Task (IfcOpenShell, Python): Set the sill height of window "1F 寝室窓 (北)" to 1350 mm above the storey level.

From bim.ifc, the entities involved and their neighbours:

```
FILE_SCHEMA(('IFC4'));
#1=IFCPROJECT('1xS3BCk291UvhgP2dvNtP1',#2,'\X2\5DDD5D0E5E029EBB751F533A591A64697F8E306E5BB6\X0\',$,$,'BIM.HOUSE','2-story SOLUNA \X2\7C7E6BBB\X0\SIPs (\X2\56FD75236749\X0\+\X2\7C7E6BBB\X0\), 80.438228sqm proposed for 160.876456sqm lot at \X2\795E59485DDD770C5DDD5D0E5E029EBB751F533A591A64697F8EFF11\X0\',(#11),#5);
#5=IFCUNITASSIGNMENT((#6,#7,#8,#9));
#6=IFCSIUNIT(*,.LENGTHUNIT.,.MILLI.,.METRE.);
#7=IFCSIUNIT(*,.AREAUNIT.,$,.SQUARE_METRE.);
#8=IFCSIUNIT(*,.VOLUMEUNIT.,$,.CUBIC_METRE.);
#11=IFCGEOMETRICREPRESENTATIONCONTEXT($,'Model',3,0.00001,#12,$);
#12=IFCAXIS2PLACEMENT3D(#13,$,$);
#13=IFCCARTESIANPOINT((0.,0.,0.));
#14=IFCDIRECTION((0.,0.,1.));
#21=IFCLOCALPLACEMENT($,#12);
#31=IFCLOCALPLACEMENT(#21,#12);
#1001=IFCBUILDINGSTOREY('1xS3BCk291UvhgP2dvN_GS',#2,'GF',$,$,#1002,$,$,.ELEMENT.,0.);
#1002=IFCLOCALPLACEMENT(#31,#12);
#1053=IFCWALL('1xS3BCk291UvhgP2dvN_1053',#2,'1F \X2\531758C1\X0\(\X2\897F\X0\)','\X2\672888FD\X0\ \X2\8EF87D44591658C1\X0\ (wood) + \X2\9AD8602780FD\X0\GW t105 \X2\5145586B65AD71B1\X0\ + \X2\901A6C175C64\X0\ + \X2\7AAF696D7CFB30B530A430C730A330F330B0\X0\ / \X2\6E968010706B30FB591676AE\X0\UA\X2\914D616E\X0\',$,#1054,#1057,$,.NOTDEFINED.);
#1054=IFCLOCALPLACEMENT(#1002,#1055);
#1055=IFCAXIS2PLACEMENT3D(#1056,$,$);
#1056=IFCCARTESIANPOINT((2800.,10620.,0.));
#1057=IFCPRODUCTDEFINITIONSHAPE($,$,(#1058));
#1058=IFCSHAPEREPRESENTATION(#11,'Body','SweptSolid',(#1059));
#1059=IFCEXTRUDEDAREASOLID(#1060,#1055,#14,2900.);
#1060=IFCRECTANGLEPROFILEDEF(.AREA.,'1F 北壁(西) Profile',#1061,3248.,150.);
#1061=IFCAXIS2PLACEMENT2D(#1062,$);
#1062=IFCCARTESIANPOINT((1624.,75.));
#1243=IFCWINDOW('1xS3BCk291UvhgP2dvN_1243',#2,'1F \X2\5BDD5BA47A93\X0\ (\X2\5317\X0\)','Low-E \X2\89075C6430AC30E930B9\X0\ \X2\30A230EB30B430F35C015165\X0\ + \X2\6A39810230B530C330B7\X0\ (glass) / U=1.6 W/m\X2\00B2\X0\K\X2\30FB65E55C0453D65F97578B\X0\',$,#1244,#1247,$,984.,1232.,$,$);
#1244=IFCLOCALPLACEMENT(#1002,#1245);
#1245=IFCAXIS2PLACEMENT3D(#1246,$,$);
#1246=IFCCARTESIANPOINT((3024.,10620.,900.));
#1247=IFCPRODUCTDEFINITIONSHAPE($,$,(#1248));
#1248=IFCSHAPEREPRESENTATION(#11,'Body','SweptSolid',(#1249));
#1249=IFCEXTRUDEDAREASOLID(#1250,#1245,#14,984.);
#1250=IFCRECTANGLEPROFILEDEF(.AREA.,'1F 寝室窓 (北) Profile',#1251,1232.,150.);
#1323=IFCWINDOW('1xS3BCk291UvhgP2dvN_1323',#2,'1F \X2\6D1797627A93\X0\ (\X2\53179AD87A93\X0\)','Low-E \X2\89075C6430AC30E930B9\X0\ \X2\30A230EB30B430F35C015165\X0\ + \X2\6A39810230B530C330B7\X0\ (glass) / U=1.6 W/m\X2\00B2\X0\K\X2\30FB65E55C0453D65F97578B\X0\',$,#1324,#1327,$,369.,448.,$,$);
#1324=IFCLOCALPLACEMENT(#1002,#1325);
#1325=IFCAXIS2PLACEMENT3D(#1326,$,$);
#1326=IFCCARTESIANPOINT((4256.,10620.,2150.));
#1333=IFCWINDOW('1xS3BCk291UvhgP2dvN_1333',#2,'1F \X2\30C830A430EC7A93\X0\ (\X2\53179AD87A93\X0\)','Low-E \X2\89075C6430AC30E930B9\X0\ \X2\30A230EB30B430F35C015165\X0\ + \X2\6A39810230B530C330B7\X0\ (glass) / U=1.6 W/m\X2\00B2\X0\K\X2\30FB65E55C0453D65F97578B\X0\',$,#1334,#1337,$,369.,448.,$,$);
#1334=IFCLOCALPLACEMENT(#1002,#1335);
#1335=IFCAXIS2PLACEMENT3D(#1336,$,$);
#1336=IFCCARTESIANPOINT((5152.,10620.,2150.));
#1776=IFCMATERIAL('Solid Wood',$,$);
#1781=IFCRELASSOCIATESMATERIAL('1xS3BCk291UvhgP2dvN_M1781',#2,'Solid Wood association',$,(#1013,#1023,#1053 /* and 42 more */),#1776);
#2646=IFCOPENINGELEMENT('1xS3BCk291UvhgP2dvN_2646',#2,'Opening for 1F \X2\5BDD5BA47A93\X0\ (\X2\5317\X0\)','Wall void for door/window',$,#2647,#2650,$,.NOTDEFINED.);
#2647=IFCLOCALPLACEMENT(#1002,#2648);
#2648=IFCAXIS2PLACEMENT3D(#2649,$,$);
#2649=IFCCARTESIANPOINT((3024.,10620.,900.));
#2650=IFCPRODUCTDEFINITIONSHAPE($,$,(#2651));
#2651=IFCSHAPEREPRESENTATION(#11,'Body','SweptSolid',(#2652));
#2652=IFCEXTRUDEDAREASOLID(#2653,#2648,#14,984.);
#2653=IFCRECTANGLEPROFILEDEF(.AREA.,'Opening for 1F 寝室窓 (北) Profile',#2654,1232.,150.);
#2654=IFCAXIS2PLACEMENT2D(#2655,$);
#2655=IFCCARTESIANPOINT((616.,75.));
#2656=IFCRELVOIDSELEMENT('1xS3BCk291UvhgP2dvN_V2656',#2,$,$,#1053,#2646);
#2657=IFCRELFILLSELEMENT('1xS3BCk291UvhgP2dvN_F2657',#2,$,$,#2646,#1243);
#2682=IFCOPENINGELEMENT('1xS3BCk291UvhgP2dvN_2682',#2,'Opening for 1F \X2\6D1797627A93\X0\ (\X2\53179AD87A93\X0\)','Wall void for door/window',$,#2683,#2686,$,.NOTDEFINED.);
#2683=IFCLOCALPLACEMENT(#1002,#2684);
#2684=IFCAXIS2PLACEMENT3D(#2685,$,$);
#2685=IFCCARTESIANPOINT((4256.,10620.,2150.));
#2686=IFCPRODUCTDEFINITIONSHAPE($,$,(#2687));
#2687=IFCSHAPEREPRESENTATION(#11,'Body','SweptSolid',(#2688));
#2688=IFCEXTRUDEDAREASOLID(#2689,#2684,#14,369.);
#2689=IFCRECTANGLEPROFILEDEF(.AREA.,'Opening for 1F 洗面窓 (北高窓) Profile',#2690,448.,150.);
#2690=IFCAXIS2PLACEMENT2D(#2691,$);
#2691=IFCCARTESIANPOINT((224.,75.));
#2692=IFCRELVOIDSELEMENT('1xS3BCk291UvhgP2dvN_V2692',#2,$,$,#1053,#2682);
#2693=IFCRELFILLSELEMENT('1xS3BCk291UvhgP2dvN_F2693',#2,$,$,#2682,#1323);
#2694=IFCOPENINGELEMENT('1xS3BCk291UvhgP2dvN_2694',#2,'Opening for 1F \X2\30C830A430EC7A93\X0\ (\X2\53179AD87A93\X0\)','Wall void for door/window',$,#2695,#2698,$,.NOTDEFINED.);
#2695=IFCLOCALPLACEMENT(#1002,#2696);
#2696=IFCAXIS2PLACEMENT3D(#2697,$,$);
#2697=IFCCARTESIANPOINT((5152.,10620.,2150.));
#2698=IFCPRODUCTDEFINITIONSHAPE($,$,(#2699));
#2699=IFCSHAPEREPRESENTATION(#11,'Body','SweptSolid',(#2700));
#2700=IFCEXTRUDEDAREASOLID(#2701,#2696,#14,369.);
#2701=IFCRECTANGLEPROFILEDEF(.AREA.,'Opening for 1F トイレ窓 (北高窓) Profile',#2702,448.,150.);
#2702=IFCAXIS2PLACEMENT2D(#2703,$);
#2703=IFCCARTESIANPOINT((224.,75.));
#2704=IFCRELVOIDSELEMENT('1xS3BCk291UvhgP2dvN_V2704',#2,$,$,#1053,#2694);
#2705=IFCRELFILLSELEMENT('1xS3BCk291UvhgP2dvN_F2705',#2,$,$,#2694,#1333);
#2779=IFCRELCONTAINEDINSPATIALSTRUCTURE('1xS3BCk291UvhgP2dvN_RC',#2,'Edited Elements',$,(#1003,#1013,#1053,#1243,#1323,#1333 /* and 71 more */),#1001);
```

```python
import numpy as np
import ifcopenshell
import ifcopenshell.api.geometry
import ifcopenshell.geom
import ifcopenshell.util.element
import ifcopenshell.util.placement
import ifcopenshell.util.shape
import ifcopenshell.util.unit

model = ifcopenshell.open("bim.ifc")
unit_scale = ifcopenshell.util.unit.calculate_unit_scale(model)

window = model.by_id(1243)
opening = window.FillsVoids[0].RelatingOpeningElement
storey = ifcopenshell.util.element.get_container(window, ifc_class="IfcBuildingStorey")
level = ifcopenshell.util.placement.get_local_placement(storey.ObjectPlacement)[2, 3]

# The opening's origin need not be at the sill, so measure its lowest point.
shape = ifcopenshell.geom.create_shape(ifcopenshell.geom.settings(), opening)
bottom = ifcopenshell.util.shape.get_shape_bottom_elevation(shape, shape.geometry) / unit_scale
dz = level + 1.35 / unit_scale - bottom

shift = np.array([0.0, 0.0, dz])
# The window is not placed relative to its opening, so move both.
for product in (opening, window):
    matrix = ifcopenshell.util.placement.get_local_placement(product.ObjectPlacement)
    matrix[:3, 3] += shift
    ifcopenshell.api.geometry.edit_object_placement(model, product=product, matrix=matrix, is_si=False)

print(f"moved by {dz * unit_scale:+.3f} m")

model.write("bim_updated.ifc")
```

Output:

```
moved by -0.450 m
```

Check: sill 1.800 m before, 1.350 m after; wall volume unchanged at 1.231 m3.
